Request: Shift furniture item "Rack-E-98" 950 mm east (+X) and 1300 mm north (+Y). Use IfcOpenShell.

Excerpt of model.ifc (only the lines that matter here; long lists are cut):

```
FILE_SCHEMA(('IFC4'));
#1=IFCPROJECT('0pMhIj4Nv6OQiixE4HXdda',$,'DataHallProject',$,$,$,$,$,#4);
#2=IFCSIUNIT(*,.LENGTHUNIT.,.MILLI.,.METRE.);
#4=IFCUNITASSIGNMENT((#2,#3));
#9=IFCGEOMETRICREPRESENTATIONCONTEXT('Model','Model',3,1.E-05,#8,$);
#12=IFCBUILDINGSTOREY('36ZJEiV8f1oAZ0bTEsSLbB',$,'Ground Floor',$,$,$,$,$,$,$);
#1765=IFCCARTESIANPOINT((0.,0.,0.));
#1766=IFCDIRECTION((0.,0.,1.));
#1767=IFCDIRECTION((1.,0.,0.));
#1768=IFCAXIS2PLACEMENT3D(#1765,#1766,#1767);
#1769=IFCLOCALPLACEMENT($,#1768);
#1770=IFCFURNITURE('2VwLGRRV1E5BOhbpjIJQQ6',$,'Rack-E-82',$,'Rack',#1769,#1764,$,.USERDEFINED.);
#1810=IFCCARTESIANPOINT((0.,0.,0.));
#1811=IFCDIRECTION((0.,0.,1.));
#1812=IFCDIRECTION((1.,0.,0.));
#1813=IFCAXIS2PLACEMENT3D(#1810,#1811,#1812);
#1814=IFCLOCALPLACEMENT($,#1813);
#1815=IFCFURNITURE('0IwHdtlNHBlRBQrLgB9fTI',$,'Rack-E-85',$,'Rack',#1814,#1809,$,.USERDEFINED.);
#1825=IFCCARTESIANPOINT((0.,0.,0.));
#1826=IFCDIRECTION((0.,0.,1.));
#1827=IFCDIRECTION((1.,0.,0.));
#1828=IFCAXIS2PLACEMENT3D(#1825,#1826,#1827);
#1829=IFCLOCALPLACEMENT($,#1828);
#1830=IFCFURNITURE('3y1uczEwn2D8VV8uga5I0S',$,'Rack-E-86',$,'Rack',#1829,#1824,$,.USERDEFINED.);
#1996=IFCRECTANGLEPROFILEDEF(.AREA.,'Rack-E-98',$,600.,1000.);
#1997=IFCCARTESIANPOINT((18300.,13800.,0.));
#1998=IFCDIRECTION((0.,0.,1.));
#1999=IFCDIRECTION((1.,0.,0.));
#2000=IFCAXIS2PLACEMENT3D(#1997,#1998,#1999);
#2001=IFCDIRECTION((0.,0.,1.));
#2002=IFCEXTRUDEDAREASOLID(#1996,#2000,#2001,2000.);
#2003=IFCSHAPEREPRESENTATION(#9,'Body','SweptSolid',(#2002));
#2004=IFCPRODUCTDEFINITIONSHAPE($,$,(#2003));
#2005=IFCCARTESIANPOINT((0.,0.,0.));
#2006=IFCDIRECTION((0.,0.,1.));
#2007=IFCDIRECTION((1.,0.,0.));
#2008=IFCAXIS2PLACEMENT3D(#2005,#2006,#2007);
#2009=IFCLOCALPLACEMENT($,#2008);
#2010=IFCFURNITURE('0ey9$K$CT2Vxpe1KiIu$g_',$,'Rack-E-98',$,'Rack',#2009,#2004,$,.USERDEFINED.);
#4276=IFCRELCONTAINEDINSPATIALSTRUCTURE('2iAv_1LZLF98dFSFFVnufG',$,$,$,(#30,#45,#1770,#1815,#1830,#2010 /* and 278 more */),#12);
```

```python
import ifcopenshell
import ifcopenshell.api.geometry
import ifcopenshell.util.placement
import ifcopenshell.util.unit

model = ifcopenshell.open("model.ifc")
unit_scale = ifcopenshell.util.unit.calculate_unit_scale(model)

item = model.by_id(2010)
matrix = ifcopenshell.util.placement.get_local_placement(item.ObjectPlacement)
matrix[0, 3] += 0.95 / unit_scale
matrix[1, 3] += 1.3 / unit_scale
ifcopenshell.api.geometry.edit_object_placement(model, product=item, matrix=matrix, is_si=False)

print(ifcopenshell.util.placement.get_local_placement(item.ObjectPlacement).round(3) + 0.0)

model.write("model-out.ifc")
```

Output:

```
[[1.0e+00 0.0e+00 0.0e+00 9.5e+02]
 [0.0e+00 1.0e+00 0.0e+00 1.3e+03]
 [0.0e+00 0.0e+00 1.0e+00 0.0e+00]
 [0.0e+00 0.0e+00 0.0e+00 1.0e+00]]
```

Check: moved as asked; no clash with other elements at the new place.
